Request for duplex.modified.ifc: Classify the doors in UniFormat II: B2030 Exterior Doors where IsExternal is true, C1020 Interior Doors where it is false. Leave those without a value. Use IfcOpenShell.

First a look at what the model holds.

```python
import ifcopenshell
import ifcopenshell.util.element

model = ifcopenshell.open("duplex.modified.ifc")
print(model.schema)
print("classifications:", [c.Name for c in model.by_type("IfcClassification")])
values = [ifcopenshell.util.element.get_pset(e, "Pset_DoorCommon", "IsExternal") for e in model.by_type("IfcDoor")]
for value in (True, False, None):
    print("IsExternal", value, values.count(value))
```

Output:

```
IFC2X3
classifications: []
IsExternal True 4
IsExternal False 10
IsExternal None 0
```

```python
import ifcopenshell
import ifcopenshell.api.classification
import ifcopenshell.util.element

model = ifcopenshell.open("duplex.modified.ifc")

# IFC2X3 requires Source and Edition and has no link from the project to the system.
system = model.create_entity("IfcClassification", Source="ASTM", Edition="E1557", Name="UniFormat II")

doors = model.by_type("IfcDoor")
external = {e: ifcopenshell.util.element.get_pset(e, "Pset_DoorCommon", "IsExternal") for e in doors}
for flag, code, name in ((True, "B2030", "Exterior Doors"), (False, "C1020", "Interior Doors")):
    products = [e for e in doors if external[e] is flag]
    ifcopenshell.api.classification.add_reference(
        model, products=products, classification=system, identification=code, name=name
    )
    print(code, len(products))

model.write("duplex.modified_edited.ifc")
```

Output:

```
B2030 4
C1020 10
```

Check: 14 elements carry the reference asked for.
